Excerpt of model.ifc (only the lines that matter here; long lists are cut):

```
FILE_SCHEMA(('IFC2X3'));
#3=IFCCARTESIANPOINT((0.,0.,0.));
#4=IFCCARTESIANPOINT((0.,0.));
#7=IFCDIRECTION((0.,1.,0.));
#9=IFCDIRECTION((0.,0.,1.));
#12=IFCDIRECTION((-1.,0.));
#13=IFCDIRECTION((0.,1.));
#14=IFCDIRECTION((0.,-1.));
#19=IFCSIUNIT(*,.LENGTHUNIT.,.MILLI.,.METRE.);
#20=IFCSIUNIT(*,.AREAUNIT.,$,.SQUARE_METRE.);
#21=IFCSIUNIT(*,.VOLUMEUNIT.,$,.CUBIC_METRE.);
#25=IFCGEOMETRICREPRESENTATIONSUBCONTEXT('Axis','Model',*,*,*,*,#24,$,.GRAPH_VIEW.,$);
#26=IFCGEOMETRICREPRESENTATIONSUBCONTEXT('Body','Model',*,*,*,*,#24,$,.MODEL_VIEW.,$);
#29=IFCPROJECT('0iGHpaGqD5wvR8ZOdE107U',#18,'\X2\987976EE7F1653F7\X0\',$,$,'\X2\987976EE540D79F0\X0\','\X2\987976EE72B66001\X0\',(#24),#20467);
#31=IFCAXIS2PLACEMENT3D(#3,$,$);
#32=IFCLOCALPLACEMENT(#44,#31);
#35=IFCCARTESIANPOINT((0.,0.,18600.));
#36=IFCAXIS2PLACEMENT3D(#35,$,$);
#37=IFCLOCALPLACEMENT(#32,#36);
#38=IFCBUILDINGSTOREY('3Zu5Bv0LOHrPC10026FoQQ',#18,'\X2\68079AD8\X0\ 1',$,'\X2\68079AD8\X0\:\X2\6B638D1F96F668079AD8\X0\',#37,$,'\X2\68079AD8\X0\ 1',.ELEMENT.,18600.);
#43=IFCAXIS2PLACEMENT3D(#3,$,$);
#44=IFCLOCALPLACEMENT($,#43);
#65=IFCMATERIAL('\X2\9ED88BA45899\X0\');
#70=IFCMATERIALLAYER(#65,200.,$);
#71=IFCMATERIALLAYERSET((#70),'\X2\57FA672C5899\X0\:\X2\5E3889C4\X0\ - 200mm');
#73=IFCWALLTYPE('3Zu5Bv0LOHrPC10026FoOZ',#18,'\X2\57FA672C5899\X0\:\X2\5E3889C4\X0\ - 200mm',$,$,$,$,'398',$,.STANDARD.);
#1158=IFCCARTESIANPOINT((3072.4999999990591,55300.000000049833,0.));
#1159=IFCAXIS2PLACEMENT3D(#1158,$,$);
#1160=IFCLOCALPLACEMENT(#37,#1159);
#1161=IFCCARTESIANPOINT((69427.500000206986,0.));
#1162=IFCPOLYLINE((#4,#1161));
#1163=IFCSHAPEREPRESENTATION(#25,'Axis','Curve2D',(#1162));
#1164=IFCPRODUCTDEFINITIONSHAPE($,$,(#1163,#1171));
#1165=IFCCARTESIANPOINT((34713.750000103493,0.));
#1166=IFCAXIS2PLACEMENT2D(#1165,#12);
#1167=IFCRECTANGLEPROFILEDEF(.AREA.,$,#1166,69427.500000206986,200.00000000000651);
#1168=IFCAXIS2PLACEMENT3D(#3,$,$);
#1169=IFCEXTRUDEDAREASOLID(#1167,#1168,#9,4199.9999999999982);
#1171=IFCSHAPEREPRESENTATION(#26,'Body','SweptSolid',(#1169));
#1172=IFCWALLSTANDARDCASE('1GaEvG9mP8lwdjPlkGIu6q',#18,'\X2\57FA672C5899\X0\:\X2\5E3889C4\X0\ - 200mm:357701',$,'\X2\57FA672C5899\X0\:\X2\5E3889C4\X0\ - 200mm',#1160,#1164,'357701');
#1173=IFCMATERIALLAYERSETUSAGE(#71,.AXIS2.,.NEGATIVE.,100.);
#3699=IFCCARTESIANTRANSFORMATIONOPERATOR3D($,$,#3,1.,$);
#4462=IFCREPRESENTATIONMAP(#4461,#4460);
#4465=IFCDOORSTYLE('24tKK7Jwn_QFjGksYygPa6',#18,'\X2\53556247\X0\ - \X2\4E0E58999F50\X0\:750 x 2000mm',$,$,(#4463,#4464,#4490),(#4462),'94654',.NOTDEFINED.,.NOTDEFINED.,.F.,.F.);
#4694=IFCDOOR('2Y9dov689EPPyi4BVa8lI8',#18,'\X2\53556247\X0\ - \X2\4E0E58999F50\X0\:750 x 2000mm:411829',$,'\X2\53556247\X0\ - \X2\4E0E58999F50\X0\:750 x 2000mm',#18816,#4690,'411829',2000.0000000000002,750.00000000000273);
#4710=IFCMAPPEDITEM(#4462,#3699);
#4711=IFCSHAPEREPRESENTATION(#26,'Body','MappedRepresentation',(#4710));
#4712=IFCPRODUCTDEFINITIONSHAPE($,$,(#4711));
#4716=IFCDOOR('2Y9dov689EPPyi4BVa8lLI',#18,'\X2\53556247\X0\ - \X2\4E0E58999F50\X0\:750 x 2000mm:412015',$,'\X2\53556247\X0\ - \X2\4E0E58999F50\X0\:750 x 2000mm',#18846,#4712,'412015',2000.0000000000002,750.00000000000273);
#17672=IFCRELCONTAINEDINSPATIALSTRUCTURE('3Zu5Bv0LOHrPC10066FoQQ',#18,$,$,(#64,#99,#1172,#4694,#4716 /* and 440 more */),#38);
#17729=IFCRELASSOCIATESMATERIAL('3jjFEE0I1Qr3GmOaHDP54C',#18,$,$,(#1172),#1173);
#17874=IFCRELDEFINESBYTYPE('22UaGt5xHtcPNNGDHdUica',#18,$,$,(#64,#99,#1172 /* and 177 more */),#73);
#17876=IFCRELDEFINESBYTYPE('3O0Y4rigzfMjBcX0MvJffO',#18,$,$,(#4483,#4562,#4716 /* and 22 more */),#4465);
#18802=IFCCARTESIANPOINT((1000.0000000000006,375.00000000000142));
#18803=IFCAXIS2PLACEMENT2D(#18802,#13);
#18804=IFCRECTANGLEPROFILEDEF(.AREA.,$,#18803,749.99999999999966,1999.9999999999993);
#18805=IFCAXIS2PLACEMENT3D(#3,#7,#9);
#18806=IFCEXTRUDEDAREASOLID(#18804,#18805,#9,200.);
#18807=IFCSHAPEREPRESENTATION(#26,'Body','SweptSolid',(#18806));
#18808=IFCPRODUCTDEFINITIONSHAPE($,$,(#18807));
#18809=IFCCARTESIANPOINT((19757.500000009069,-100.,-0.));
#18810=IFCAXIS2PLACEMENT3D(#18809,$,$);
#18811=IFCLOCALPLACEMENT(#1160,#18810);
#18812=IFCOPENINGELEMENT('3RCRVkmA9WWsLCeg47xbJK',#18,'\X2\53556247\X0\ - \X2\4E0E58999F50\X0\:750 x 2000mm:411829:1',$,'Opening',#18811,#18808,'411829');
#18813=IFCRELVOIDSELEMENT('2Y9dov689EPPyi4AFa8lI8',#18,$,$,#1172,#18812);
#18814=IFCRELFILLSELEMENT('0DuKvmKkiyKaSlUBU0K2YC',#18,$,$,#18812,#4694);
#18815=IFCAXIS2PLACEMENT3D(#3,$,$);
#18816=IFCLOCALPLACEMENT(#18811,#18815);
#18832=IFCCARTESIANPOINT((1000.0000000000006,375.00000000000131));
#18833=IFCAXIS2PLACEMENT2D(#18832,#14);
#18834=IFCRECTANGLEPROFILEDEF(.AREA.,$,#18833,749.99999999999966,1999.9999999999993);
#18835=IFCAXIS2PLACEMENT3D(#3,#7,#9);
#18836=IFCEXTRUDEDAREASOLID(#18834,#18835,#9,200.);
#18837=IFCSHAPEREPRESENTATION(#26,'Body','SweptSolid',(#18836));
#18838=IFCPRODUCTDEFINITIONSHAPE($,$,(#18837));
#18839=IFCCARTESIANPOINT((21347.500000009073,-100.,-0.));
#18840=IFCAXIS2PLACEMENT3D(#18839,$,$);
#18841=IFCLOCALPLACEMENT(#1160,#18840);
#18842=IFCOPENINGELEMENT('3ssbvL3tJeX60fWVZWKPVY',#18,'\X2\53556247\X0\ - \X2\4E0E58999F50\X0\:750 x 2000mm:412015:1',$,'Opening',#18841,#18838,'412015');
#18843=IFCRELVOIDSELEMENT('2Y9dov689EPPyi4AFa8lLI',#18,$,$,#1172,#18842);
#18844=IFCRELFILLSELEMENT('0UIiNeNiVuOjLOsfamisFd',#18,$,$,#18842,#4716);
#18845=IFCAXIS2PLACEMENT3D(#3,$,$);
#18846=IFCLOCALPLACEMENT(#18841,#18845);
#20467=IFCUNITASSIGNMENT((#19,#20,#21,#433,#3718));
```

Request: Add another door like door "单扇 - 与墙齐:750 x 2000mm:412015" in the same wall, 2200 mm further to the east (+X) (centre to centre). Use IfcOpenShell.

```python
import ifcopenshell
import ifcopenshell.api.feature
import ifcopenshell.api.geometry
import ifcopenshell.api.root
import ifcopenshell.geom
import ifcopenshell.util.element
import ifcopenshell.util.placement
import ifcopenshell.util.shape
import ifcopenshell.util.unit

model = ifcopenshell.open("model.ifc")
unit_scale = ifcopenshell.util.unit.calculate_unit_scale(model)
settings = ifcopenshell.geom.settings()


def volume(element):
    """Net volume in cubic metres, openings subtracted."""
    shape = ifcopenshell.geom.create_shape(settings, element)
    return ifcopenshell.util.shape.get_volume(shape.geometry)


def reuse_history(source, copy):
    """copy_class also copies each property set's owner history, people and application; keep the originals."""
    for rel in copy.IsDefinedBy:
        if rel.is_a("IfcRelDefinesByProperties") and (history := rel.RelatingPropertyDefinition.OwnerHistory):
            rel.RelatingPropertyDefinition.OwnerHistory = source.OwnerHistory
            ifcopenshell.util.element.remove_deep2(model, history)


door = model.by_id(4716)
opening = door.FillsVoids[0].RelatingOpeningElement
wall = opening.VoidsElements[0].RelatingBuildingElement
before = volume(wall)
shift = ifcopenshell.util.placement.get_local_placement(wall.ObjectPlacement)[:3, 0] * 2.2 / unit_scale

# copy_class copies the void relationship, type, container and properties, but no geometry.
new_opening = ifcopenshell.api.root.copy_class(model, product=opening)
new_opening.Representation = ifcopenshell.util.element.copy_deep(
    model, opening.Representation, exclude=["IfcGeometricRepresentationContext", "IfcRepresentationMap"]
)
new_opening.Name = "单扇 - 与墙齐:750 x 2000mm"
new_opening.Tag = None
new_door = ifcopenshell.api.root.copy_class(model, product=door)
new_door.Representation = ifcopenshell.util.element.copy_deep(
    model, door.Representation, exclude=["IfcGeometricRepresentationContext", "IfcRepresentationMap"]
)
new_door.Name = "单扇 - 与墙齐:750 x 2000mm"
new_door.Tag = None
reuse_history(door, new_door)
fills = ifcopenshell.api.feature.add_filling(model, opening=new_opening, element=new_door)
fills.OwnerHistory = new_door.OwnerHistory  # required in IFC2X3

for old, new in ((opening, new_opening), (door, new_door)):
    matrix = ifcopenshell.util.placement.get_local_placement(old.ObjectPlacement)
    matrix[:3, 3] += shift
    ifcopenshell.api.geometry.edit_object_placement(model, product=new, matrix=matrix, is_si=False)

after = volume(wall)

print(f"wall volume {before:.3f} -> {after:.3f} m3")

model.write("model_updated.ifc")
```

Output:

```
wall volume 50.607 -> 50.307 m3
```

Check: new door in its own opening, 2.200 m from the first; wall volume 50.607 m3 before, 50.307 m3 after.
